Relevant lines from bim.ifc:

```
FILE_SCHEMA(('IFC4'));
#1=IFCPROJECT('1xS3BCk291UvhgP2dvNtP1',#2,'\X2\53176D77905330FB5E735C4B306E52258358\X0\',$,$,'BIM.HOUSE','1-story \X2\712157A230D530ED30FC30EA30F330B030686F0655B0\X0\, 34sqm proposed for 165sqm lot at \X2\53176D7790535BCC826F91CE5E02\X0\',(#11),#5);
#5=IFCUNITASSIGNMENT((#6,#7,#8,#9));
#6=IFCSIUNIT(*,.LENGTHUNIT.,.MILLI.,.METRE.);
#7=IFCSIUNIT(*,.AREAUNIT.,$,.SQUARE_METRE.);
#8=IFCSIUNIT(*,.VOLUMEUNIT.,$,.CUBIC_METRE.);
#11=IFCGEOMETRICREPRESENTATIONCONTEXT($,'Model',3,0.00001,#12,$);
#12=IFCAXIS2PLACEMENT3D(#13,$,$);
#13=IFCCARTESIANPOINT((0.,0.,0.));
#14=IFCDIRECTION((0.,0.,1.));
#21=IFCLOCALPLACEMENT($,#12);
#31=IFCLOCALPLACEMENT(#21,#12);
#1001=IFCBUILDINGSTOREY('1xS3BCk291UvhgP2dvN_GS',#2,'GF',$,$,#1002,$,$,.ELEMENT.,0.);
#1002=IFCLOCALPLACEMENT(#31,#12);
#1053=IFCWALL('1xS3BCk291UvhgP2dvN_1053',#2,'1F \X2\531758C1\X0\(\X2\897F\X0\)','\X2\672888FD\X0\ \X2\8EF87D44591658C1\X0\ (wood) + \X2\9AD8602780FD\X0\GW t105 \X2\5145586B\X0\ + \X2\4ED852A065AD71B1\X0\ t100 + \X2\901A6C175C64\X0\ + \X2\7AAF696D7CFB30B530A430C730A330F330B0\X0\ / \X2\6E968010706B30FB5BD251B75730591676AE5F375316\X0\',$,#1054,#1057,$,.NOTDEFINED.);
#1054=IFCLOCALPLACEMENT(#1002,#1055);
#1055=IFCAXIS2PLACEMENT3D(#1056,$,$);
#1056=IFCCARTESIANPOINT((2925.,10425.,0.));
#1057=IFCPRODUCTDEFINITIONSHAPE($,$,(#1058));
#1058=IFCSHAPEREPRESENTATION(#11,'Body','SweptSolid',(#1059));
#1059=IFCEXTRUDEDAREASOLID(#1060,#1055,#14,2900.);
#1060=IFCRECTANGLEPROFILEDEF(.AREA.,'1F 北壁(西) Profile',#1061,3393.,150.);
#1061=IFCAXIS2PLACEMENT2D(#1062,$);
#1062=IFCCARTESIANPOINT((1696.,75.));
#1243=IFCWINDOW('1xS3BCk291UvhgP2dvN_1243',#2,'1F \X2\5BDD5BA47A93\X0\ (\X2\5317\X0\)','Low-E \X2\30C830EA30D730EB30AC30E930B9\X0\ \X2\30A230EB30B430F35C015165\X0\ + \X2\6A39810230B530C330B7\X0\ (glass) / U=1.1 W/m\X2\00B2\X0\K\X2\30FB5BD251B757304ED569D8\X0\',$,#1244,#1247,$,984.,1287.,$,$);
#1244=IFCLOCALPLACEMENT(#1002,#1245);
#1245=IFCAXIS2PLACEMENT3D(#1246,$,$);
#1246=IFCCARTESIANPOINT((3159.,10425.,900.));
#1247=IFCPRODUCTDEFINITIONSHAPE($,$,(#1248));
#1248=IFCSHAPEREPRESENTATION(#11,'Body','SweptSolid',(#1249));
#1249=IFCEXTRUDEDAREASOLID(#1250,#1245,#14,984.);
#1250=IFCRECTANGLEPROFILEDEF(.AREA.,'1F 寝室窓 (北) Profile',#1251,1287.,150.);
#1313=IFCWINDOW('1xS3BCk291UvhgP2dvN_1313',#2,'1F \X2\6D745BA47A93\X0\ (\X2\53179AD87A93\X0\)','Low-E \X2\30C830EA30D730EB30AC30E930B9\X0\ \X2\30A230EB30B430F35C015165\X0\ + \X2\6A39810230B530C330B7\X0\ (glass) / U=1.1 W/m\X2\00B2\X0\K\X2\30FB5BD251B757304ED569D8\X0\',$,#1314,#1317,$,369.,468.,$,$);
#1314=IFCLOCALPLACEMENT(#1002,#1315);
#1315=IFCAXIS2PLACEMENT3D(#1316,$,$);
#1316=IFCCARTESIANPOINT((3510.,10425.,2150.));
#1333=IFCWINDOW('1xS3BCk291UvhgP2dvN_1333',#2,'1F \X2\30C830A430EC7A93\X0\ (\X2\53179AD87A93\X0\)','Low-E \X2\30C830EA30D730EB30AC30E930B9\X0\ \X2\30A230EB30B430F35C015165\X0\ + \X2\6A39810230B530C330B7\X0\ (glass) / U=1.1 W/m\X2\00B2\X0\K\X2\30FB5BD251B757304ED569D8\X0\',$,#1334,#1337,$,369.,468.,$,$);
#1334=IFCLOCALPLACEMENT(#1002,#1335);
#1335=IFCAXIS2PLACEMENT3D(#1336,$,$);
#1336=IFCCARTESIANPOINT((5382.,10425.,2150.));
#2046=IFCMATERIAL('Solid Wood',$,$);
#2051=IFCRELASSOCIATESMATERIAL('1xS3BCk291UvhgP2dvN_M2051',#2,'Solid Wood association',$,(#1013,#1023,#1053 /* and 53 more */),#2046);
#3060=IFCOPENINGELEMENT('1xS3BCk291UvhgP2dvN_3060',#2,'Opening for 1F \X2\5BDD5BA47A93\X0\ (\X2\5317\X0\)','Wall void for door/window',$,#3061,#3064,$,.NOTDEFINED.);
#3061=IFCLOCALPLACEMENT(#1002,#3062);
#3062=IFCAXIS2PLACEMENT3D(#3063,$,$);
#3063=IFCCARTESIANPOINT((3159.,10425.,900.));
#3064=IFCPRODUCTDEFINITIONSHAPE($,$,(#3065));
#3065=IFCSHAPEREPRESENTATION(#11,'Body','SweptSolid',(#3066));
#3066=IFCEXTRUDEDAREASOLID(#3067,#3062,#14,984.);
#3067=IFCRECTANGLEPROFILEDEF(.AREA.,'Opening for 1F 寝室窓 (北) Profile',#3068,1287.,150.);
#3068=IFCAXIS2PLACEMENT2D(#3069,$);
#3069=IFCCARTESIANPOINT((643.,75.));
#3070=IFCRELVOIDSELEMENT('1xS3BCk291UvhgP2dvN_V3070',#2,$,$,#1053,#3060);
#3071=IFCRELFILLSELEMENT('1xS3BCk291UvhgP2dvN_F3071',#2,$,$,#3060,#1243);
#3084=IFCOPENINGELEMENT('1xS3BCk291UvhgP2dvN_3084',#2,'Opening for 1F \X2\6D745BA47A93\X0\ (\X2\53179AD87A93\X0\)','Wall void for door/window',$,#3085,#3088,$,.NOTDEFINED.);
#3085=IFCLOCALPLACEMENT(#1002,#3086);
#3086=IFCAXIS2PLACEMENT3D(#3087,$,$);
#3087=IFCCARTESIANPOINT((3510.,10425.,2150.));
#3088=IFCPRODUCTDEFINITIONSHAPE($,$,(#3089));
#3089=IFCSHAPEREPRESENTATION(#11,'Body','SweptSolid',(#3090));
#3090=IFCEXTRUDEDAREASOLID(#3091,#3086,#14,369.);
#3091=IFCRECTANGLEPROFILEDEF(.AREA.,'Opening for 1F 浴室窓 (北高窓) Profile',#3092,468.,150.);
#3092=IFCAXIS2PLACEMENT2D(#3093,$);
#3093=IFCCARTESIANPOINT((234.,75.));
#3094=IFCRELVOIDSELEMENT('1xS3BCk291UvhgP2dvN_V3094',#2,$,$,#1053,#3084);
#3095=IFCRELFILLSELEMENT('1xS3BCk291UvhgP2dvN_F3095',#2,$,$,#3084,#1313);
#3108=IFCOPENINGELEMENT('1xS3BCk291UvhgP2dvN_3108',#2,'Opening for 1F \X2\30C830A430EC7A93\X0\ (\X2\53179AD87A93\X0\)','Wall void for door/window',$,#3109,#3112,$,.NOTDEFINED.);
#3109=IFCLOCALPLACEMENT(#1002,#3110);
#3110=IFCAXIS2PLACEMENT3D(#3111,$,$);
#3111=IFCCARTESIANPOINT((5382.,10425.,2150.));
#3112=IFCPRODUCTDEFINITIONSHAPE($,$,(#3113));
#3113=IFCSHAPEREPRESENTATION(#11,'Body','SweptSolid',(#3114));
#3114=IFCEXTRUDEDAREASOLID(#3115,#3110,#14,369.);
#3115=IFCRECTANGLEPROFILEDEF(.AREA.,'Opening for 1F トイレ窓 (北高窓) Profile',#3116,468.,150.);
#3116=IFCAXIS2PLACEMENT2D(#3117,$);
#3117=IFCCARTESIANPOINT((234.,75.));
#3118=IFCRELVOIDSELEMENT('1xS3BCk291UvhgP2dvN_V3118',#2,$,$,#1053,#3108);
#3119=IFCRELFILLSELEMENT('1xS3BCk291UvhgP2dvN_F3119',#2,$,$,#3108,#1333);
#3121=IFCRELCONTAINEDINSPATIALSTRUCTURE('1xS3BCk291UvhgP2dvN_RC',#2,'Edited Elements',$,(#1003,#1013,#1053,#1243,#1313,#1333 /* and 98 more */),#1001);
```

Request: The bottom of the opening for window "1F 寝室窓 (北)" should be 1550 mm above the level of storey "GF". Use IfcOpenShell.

```python
import numpy as np
import ifcopenshell
import ifcopenshell.api.geometry
import ifcopenshell.geom
import ifcopenshell.util.element
import ifcopenshell.util.placement
import ifcopenshell.util.shape
import ifcopenshell.util.unit

model = ifcopenshell.open("bim.ifc")
unit_scale = ifcopenshell.util.unit.calculate_unit_scale(model)

window = model.by_guid("1xS3BCk291UvhgP2dvN_1243")
opening = window.FillsVoids[0].RelatingOpeningElement
storey = ifcopenshell.util.element.get_container(window, ifc_class="IfcBuildingStorey")
level = ifcopenshell.util.placement.get_local_placement(storey.ObjectPlacement)[2, 3]

# The opening's origin need not be at the sill, so measure its lowest point.
shape = ifcopenshell.geom.create_shape(ifcopenshell.geom.settings(), opening)
bottom = ifcopenshell.util.shape.get_shape_bottom_elevation(shape, shape.geometry) / unit_scale
dz = level + 1.55 / unit_scale - bottom

shift = np.array([0.0, 0.0, dz])
# The window is not placed relative to its opening, so move both.
for product in (opening, window):
    matrix = ifcopenshell.util.placement.get_local_placement(product.ObjectPlacement)
    matrix[:3, 3] += shift
    ifcopenshell.api.geometry.edit_object_placement(model, product=product, matrix=matrix, is_si=False)

print(f"moved by {dz * unit_scale:+.3f} m")

model.write("bim-out.ifc")
```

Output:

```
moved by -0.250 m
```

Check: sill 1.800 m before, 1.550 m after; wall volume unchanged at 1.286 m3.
